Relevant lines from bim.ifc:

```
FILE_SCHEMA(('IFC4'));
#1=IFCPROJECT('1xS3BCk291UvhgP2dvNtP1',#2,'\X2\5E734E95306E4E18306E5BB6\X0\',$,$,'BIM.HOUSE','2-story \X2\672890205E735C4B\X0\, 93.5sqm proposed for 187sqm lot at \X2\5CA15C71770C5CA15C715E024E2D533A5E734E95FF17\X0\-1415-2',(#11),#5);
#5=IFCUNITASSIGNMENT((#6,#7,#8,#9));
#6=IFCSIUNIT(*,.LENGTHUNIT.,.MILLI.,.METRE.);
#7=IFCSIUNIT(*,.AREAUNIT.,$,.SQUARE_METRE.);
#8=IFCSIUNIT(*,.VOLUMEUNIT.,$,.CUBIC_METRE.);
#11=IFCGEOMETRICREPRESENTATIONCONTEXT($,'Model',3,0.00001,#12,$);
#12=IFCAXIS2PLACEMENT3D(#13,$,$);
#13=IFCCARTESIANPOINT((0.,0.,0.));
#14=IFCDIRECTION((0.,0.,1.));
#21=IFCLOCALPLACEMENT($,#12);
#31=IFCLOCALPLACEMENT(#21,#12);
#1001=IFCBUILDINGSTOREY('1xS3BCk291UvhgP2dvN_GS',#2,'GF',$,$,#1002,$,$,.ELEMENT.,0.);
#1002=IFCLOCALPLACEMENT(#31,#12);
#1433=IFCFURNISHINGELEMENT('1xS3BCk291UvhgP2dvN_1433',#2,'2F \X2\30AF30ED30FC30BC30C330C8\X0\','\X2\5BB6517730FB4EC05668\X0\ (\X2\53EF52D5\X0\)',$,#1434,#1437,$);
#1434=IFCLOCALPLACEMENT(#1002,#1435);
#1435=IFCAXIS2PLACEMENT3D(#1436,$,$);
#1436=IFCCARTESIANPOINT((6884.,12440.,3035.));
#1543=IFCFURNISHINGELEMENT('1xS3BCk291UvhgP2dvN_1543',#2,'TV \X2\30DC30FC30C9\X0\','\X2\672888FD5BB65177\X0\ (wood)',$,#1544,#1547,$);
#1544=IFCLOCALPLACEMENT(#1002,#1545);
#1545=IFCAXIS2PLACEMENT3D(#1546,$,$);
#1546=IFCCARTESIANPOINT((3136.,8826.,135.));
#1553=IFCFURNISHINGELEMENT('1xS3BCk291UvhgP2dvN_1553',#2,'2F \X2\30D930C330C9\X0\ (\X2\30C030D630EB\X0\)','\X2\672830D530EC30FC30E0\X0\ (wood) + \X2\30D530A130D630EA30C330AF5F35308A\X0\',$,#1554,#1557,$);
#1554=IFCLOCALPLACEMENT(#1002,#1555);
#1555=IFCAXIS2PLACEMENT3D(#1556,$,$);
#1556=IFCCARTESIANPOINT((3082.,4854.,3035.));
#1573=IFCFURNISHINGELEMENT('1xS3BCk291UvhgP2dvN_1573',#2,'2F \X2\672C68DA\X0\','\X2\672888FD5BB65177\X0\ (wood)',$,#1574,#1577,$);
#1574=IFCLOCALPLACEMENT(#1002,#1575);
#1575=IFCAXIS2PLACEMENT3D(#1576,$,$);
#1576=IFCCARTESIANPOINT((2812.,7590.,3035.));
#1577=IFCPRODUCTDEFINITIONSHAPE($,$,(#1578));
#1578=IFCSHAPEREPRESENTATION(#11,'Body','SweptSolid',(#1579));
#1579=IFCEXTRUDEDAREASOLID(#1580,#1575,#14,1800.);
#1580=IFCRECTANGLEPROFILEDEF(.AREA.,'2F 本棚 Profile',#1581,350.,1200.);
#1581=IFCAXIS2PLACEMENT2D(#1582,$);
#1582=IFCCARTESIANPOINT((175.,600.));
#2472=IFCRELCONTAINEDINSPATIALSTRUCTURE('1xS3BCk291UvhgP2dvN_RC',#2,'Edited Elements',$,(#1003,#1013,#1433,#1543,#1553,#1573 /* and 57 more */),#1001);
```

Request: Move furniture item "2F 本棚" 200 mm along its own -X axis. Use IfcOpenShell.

```python
import ifcopenshell
import ifcopenshell.api.geometry
import ifcopenshell.util.placement
import ifcopenshell.util.unit

model = ifcopenshell.open("bim.ifc")
unit_scale = ifcopenshell.util.unit.calculate_unit_scale(model)

item = model.by_id(1573)
matrix = ifcopenshell.util.placement.get_local_placement(item.ObjectPlacement)
matrix[:3, 3] -= matrix[:3, 0] * 0.2 / unit_scale
ifcopenshell.api.geometry.edit_object_placement(model, product=item, matrix=matrix, is_si=False)

print(ifcopenshell.util.placement.get_local_placement(item.ObjectPlacement).round(3) + 0.0)

model.write("bim_rev.ifc")
```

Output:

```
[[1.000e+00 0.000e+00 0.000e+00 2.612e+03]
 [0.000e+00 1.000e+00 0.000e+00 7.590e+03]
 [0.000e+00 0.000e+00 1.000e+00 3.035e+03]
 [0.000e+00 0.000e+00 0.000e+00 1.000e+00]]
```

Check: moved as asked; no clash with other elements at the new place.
